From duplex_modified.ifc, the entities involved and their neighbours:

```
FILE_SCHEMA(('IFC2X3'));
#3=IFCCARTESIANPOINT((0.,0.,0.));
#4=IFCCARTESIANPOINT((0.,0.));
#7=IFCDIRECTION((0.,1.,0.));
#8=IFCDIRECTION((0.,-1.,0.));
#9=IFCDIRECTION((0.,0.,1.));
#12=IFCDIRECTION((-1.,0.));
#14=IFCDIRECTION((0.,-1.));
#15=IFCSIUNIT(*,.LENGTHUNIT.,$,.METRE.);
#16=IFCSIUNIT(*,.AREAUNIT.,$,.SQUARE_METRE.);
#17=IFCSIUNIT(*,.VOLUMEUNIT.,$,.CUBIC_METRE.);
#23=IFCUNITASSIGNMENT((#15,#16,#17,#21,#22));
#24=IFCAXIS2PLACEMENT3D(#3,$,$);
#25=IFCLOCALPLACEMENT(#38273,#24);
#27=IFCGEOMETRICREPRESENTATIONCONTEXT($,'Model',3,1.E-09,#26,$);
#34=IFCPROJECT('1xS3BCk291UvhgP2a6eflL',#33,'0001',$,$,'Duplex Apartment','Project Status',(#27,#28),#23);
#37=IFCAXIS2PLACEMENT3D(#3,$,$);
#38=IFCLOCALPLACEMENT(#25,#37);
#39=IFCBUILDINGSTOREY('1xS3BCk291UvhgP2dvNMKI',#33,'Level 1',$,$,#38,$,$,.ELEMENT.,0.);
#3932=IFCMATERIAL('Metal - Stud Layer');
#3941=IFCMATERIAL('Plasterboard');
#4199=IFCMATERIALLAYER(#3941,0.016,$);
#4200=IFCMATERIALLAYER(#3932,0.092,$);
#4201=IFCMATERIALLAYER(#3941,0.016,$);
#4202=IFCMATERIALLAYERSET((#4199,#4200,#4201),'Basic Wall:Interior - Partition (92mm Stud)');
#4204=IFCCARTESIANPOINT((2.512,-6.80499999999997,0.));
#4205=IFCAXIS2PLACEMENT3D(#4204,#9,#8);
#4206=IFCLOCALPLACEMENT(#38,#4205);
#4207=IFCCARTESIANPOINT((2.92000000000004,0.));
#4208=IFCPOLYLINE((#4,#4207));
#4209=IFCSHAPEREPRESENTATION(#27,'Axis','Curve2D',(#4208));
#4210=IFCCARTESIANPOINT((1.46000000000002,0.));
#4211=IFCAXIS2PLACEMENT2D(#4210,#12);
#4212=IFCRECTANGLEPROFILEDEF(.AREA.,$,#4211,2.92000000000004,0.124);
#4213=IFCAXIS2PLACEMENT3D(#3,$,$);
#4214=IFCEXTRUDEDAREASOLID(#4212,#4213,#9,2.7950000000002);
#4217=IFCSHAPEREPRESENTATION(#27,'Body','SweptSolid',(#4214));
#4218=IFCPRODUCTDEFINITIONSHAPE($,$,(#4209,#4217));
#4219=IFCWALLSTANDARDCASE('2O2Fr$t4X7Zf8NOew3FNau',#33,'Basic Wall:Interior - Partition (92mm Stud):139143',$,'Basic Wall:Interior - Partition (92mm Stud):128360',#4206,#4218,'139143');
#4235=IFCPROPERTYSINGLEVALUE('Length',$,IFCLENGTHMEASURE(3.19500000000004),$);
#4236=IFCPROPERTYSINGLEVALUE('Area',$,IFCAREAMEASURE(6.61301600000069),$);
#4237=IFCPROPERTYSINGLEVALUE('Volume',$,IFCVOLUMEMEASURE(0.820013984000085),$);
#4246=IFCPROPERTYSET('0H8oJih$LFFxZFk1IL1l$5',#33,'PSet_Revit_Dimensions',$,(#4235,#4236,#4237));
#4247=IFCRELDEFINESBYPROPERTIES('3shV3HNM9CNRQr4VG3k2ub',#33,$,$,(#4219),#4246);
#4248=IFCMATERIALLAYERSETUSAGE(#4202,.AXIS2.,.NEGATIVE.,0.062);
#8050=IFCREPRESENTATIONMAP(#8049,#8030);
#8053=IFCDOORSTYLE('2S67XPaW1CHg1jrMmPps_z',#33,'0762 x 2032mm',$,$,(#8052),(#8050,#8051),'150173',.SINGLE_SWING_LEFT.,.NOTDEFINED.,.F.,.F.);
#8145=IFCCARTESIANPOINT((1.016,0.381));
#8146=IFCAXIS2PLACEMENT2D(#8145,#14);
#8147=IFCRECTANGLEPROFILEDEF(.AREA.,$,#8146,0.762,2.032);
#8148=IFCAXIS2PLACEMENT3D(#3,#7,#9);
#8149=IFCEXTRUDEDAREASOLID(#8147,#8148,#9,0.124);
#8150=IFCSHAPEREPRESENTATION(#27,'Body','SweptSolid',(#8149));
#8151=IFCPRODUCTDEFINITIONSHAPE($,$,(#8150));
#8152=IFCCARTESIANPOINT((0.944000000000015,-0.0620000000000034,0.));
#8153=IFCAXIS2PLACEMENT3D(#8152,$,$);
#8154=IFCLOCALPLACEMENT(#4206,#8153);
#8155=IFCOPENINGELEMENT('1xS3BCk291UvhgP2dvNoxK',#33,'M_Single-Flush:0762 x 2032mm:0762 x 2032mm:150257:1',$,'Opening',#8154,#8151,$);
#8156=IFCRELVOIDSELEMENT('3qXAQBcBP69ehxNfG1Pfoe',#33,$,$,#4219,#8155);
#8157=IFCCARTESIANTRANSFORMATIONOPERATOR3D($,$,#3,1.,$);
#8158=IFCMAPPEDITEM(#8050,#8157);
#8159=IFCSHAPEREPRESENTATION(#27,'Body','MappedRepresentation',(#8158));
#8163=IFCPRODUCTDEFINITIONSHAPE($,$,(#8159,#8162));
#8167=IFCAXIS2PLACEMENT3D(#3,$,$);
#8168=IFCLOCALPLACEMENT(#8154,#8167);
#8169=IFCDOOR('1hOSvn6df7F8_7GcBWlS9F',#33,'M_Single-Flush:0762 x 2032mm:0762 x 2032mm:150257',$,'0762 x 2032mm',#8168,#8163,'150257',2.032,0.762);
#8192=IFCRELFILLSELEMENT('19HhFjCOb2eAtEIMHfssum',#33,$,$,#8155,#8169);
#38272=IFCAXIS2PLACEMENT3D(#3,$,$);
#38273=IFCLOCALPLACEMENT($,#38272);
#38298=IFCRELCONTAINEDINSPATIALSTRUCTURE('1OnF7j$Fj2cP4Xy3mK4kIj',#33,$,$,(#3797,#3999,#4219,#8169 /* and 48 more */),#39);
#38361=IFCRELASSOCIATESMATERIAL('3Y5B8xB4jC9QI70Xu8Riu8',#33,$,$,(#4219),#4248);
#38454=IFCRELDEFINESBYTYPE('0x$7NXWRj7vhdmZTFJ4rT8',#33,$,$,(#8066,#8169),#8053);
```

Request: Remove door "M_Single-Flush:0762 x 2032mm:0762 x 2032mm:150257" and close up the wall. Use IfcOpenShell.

```python
import ifcopenshell
import ifcopenshell.api.feature
import ifcopenshell.api.pset
import ifcopenshell.api.root
import ifcopenshell.geom
import ifcopenshell.util.element
import ifcopenshell.util.shape
import ifcopenshell.util.unit

model = ifcopenshell.open("duplex_modified.ifc")
area_scale = ifcopenshell.util.unit.calculate_unit_scale(model, "AREAUNIT")
volume_scale = ifcopenshell.util.unit.calculate_unit_scale(model, "VOLUMEUNIT")
settings = ifcopenshell.geom.settings()


def volume(element):
    """Net volume in cubic metres, openings subtracted."""
    shape = ifcopenshell.geom.create_shape(settings, element)
    return ifcopenshell.util.shape.get_volume(shape.geometry)


door = model.by_id(8169)
opening = door.FillsVoids[0].RelatingOpeningElement
wall = opening.VoidsElements[0].RelatingBuildingElement
before = volume(wall)

ifcopenshell.api.root.remove_product(model, product=door)
ifcopenshell.api.feature.remove_feature(model, feature=opening)

after = volume(wall)
thickness = 0.124  # wall thickness in metres

# Update the wall's stored quantities.
pset = model.by_id(ifcopenshell.util.element.get_pset(wall, "PSet_Revit_Dimensions", should_inherit=False)["id"])
ifcopenshell.api.pset.edit_pset(model, pset=pset, properties={
    "Area": model.create_entity("IfcAreaMeasure", after / thickness / area_scale),
    "Volume": model.create_entity("IfcVolumeMeasure", after / volume_scale),
})

print(f"wall volume {before:.3f} -> {after:.3f} m3")

model.write("duplex_modified_edited.ifc")
```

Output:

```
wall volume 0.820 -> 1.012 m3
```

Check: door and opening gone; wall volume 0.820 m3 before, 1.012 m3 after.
